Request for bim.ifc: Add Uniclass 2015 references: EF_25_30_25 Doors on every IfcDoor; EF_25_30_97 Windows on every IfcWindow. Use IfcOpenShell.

First a look at what the model holds.

```python
import ifcopenshell

model = ifcopenshell.open("bim.ifc")
print(model.schema)
print("classifications:", [c.Name for c in model.by_type("IfcClassification")])
for ifc_class in ("IfcDoor", "IfcRoof", "IfcStair", "IfcWall", "IfcWindow"):
    print(ifc_class, len(model.by_type(ifc_class)))
```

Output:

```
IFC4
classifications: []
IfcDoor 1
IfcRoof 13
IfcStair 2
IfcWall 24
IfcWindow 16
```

```python
import ifcopenshell
import ifcopenshell.api.classification

model = ifcopenshell.open("bim.ifc")

system = ifcopenshell.api.classification.add_classification(model, classification="Uniclass 2015")

codes = {
    "IfcDoor": ("EF_25_30_25", "Doors"),
    "IfcWindow": ("EF_25_30_97", "Windows"),
}
for ifc_class, (code, name) in codes.items():
    products = model.by_type(ifc_class)
    ifcopenshell.api.classification.add_reference(
        model, products=products, classification=system, identification=code, name=name
    )
    print(code, len(products))

model.write("bim_v2.ifc")
```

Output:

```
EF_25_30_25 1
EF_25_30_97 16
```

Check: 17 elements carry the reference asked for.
